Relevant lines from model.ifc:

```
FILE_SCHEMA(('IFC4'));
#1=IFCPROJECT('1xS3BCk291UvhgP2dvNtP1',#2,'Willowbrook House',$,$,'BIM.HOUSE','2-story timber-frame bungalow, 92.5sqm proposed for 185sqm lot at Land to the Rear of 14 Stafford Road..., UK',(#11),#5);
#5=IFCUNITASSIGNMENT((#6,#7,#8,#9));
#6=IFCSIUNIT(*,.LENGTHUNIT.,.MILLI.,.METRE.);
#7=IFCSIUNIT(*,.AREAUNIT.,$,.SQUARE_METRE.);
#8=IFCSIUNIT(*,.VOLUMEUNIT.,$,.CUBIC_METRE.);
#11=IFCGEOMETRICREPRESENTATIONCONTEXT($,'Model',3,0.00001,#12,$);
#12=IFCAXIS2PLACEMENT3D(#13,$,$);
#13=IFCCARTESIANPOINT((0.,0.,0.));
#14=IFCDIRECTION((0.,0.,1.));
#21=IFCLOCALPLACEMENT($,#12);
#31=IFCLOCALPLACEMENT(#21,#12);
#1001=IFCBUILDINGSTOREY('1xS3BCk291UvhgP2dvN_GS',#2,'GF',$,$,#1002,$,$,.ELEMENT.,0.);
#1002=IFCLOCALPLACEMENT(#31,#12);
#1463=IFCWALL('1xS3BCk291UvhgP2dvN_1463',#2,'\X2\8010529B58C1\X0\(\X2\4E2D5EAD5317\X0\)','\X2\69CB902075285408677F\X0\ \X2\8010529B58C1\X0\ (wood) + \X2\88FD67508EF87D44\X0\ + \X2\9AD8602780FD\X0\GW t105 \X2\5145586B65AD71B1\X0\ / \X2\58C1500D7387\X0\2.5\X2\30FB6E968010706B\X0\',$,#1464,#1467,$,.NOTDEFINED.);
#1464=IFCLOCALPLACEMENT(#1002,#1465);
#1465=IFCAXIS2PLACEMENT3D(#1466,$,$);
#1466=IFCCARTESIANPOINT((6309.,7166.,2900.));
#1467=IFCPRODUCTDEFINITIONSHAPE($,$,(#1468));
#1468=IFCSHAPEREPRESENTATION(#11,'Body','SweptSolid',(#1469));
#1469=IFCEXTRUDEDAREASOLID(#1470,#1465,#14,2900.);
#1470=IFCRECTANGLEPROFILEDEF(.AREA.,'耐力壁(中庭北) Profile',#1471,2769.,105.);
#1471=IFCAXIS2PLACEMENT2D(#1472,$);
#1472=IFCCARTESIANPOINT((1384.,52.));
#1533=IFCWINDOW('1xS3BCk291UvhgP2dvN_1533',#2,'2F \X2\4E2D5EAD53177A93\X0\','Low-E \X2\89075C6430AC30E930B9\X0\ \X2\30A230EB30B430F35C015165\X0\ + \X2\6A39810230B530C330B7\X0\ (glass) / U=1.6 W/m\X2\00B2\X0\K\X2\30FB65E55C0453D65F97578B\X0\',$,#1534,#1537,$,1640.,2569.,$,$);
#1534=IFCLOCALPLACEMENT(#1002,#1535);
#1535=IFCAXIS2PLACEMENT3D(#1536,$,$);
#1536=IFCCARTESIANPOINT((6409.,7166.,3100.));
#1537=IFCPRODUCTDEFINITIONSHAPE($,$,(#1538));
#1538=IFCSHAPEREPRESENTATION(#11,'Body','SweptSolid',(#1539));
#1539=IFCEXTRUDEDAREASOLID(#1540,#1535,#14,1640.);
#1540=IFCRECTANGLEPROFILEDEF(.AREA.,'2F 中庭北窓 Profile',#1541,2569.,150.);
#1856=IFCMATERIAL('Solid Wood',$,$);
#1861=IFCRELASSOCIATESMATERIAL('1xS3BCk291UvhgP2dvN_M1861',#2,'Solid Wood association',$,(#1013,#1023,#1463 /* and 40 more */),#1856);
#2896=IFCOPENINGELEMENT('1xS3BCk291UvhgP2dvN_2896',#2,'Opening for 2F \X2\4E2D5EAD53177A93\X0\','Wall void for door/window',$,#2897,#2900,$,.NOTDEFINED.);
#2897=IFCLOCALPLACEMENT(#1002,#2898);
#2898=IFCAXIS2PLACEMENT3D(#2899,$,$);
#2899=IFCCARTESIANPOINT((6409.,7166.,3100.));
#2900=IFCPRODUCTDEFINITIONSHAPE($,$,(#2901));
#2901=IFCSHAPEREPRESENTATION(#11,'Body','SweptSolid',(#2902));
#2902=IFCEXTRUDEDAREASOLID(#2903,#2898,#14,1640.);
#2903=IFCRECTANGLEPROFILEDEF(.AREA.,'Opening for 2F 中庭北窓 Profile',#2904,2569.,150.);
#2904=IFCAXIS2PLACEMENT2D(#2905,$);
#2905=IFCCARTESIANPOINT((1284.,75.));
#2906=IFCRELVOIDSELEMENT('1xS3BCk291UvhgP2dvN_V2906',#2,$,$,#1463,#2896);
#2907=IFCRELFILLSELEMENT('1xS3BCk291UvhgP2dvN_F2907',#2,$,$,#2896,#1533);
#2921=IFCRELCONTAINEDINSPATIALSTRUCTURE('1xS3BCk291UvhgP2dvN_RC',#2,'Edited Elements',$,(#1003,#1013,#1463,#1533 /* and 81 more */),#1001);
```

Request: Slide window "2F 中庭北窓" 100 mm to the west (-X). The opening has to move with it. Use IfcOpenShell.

```python
import ifcopenshell
import ifcopenshell.api.geometry
import ifcopenshell.util.placement
import ifcopenshell.util.unit

model = ifcopenshell.open("model.ifc")
unit_scale = ifcopenshell.util.unit.calculate_unit_scale(model)

window = model.by_id(1533)
opening = window.FillsVoids[0].RelatingOpeningElement
wall = opening.VoidsElements[0].RelatingBuildingElement

wall_matrix = ifcopenshell.util.placement.get_local_placement(wall.ObjectPlacement)
shift = wall_matrix[:3, 0] * -0.1 / unit_scale
before = ifcopenshell.util.placement.get_local_placement(window.ObjectPlacement)[:3, 3].copy()

# The window is not placed relative to its opening, so move both.
for product in (opening, window):
    matrix = ifcopenshell.util.placement.get_local_placement(product.ObjectPlacement)
    matrix[:3, 3] += shift
    ifcopenshell.api.geometry.edit_object_placement(model, product=product, matrix=matrix, is_si=False)

after = ifcopenshell.util.placement.get_local_placement(window.ObjectPlacement)[:3, 3]
print("window moved by", (after - before).round(3) + 0.0)

model.write("model_updated.ifc")
```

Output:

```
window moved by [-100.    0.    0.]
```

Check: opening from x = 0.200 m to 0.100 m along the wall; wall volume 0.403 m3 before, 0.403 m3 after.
